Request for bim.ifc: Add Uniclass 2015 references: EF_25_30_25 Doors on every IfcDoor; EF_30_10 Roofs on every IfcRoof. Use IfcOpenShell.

First a look at what the model holds.

```python
import ifcopenshell

model = ifcopenshell.open("bim.ifc")
print(model.schema)
print("classifications:", [c.Name for c in model.by_type("IfcClassification")])
for ifc_class in ("IfcDoor", "IfcRoof", "IfcStair", "IfcWall", "IfcWindow"):
    print(ifc_class, len(model.by_type(ifc_class)))
```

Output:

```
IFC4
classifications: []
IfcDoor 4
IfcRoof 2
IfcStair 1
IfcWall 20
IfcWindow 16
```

```python
import ifcopenshell
import ifcopenshell.api.classification

model = ifcopenshell.open("bim.ifc")

system = ifcopenshell.api.classification.add_classification(model, classification="Uniclass 2015")

codes = {
    "IfcDoor": ("EF_25_30_25", "Doors"),
    "IfcRoof": ("EF_30_10", "Roofs"),
}
for ifc_class, (code, name) in codes.items():
    products = model.by_type(ifc_class)
    ifcopenshell.api.classification.add_reference(
        model, products=products, classification=system, identification=code, name=name
    )
    print(code, len(products))

model.write("bim_v2.ifc")
```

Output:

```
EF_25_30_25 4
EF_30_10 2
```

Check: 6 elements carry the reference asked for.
